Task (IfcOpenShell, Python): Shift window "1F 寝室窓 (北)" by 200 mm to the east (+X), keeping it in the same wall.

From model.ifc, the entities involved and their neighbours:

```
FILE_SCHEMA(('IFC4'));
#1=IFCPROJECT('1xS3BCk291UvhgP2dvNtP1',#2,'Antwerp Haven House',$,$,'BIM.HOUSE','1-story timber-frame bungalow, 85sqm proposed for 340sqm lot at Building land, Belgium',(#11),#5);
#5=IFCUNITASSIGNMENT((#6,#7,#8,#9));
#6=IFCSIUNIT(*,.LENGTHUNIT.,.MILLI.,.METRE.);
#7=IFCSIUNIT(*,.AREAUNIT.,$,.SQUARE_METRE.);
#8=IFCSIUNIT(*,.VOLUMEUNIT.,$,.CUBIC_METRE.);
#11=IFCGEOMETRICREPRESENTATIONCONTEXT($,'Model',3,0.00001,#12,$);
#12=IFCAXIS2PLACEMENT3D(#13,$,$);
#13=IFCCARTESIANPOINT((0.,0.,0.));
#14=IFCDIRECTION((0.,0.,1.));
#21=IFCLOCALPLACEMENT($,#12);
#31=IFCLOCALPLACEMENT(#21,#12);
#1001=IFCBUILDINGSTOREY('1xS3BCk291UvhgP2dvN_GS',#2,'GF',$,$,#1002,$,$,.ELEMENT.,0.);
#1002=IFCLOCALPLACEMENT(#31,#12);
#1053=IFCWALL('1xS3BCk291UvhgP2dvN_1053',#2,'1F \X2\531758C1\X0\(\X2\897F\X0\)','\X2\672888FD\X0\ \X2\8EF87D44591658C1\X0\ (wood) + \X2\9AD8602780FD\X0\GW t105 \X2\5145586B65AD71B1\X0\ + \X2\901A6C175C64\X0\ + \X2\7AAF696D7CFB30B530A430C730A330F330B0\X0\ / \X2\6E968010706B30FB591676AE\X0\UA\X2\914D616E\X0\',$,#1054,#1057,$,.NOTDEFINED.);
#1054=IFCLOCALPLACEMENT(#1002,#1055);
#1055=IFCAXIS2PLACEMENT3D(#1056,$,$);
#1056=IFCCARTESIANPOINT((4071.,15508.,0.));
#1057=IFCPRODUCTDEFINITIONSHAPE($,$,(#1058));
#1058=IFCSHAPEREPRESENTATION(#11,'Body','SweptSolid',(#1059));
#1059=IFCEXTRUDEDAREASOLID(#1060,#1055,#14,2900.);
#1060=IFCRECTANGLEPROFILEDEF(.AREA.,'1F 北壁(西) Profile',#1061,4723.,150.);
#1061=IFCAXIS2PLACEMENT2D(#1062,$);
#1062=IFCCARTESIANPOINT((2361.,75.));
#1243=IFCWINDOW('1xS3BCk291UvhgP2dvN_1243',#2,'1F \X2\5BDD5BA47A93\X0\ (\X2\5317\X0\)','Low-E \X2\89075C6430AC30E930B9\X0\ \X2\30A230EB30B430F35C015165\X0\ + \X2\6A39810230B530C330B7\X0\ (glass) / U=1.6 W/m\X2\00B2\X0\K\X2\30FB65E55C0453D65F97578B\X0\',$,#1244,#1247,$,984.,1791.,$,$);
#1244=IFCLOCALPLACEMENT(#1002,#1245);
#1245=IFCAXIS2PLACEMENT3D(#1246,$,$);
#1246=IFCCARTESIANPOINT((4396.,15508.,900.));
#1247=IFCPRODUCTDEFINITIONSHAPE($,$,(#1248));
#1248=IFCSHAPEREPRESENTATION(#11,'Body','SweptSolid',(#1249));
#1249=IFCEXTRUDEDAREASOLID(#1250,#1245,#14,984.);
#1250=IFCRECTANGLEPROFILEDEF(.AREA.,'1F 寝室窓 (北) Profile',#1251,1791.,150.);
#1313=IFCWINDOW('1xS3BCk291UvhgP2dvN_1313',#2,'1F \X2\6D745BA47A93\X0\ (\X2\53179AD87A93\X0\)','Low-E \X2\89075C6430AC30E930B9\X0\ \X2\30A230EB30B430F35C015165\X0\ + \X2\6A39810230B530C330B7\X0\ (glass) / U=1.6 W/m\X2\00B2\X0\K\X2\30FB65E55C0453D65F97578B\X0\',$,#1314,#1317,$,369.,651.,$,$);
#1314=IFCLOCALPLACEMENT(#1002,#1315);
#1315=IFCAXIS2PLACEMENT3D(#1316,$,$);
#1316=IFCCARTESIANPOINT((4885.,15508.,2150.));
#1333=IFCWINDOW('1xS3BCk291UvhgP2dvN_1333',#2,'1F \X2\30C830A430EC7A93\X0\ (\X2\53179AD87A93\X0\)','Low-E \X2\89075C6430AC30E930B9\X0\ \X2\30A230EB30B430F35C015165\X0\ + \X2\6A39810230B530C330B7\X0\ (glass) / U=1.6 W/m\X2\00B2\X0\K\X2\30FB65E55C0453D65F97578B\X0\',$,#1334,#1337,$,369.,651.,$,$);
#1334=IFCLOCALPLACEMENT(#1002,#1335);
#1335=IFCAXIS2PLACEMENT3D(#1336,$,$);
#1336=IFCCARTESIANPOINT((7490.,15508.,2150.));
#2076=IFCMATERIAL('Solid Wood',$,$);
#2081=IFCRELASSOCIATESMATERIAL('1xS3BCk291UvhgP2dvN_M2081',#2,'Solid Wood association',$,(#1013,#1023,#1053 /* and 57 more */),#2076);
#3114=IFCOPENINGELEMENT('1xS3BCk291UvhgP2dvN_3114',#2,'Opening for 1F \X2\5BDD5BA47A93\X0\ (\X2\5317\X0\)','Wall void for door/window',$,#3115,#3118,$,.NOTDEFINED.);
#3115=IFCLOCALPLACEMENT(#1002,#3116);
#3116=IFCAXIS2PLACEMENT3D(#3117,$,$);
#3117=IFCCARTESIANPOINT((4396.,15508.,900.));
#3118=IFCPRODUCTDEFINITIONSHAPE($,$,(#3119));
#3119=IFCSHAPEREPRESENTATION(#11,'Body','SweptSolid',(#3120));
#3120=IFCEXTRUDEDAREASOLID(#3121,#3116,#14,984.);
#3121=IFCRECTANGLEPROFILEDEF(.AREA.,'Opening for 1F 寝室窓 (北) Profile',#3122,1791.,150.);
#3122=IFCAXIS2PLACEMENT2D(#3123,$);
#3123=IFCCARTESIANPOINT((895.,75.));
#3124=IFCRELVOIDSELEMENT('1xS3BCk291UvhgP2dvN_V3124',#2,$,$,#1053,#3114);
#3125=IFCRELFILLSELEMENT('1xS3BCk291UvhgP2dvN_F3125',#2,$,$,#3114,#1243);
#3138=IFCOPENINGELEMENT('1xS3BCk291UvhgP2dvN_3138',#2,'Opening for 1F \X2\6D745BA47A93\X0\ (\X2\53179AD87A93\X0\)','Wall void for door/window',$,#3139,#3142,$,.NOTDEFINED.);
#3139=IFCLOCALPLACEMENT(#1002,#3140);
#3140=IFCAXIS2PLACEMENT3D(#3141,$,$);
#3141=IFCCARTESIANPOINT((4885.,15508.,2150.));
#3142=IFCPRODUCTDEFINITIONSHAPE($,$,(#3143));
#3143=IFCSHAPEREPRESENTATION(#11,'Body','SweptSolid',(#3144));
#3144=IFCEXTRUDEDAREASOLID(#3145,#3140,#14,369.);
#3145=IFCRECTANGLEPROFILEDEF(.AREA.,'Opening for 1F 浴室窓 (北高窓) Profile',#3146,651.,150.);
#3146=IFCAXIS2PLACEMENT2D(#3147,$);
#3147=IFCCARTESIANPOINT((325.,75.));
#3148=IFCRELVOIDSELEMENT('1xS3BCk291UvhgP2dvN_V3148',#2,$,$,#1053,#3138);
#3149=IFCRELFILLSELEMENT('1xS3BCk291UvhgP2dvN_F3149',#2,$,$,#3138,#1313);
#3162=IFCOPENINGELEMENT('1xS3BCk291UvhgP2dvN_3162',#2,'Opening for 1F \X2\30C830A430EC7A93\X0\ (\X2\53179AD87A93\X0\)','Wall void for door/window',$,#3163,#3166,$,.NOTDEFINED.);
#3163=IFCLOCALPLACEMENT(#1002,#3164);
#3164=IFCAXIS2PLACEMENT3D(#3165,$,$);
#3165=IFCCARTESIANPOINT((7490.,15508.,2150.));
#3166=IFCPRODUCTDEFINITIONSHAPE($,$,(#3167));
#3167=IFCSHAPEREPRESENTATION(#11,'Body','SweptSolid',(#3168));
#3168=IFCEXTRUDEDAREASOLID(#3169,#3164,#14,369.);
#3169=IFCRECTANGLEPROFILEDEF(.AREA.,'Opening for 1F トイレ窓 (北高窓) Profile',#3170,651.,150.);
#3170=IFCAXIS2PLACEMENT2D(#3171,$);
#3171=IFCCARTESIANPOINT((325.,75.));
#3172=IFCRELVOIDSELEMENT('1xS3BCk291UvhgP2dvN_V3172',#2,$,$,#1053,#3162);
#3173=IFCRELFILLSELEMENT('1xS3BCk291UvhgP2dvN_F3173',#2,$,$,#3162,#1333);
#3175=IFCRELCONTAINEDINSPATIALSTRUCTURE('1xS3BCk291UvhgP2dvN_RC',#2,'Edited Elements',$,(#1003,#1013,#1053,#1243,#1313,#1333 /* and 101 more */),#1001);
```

```python
import ifcopenshell
import ifcopenshell.api.geometry
import ifcopenshell.util.placement
import ifcopenshell.util.unit

model = ifcopenshell.open("model.ifc")
unit_scale = ifcopenshell.util.unit.calculate_unit_scale(model)

window = model.by_guid("1xS3BCk291UvhgP2dvN_1243")
opening = window.FillsVoids[0].RelatingOpeningElement
wall = opening.VoidsElements[0].RelatingBuildingElement

wall_matrix = ifcopenshell.util.placement.get_local_placement(wall.ObjectPlacement)
shift = wall_matrix[:3, 0] * 0.2 / unit_scale
before = ifcopenshell.util.placement.get_local_placement(window.ObjectPlacement)[:3, 3].copy()

# The window is not placed relative to its opening, so move both.
for product in (opening, window):
    matrix = ifcopenshell.util.placement.get_local_placement(product.ObjectPlacement)
    matrix[:3, 3] += shift
    ifcopenshell.api.geometry.edit_object_placement(model, product=product, matrix=matrix, is_si=False)

after = ifcopenshell.util.placement.get_local_placement(window.ObjectPlacement)[:3, 3]
print("window moved by", (after - before).round(3) + 0.0)

model.write("model_rev.ifc")
```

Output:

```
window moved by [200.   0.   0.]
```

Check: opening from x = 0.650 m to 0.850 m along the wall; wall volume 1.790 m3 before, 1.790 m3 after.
